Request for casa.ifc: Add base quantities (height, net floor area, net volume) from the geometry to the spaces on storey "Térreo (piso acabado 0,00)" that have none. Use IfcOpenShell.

First a look at what the model holds.

```python
import ifcopenshell
import ifcopenshell.util.element
import ifcopenshell.util.unit

model = ifcopenshell.open("casa.ifc")
print(model.schema)
for unit_type in ("LENGTHUNIT", "AREAUNIT", "VOLUMEUNIT"):
    print(unit_type, ifcopenshell.util.unit.calculate_unit_scale(model, unit_type))
storey = next(s for s in model.by_type("IfcBuildingStorey") if s.Name == "Térreo (piso acabado 0,00)")
spaces = [e for e in ifcopenshell.util.element.get_decomposition(storey) if e.is_a("IfcSpace")]
for e in sorted(spaces, key=lambda e: e.id()):
    print(e.id(), e.is_a(), e.Name, list(ifcopenshell.util.element.get_psets(e, qtos_only=True)), sep=" | ")
```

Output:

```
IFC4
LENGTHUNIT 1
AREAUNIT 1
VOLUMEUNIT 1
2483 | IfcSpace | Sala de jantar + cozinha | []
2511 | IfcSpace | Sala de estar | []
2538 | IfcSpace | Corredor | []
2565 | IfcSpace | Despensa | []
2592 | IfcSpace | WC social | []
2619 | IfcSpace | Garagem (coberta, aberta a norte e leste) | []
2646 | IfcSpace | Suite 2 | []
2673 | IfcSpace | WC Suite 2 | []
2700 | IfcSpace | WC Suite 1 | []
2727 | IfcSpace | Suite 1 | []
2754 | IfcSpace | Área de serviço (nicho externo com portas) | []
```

```python
import ifcopenshell
import ifcopenshell.api.pset
import ifcopenshell.geom
import ifcopenshell.util.element
import ifcopenshell.util.shape
import ifcopenshell.util.unit

model = ifcopenshell.open("casa.ifc")
unit_scale = ifcopenshell.util.unit.calculate_unit_scale(model)
area_scale = ifcopenshell.util.unit.calculate_unit_scale(model, "AREAUNIT")
volume_scale = ifcopenshell.util.unit.calculate_unit_scale(model, "VOLUMEUNIT")
settings = ifcopenshell.geom.settings()

storey = next(s for s in model.by_type("IfcBuildingStorey") if s.Name == "Térreo (piso acabado 0,00)")
spaces = [e for e in ifcopenshell.util.element.get_decomposition(storey) if e.is_a("IfcSpace")]

for e in sorted(spaces, key=lambda e: e.id()):
    if ifcopenshell.util.element.get_psets(e, qtos_only=True, should_inherit=False):
        continue
    # Geometry comes back in metres, in the element's own axes.
    shape = ifcopenshell.geom.create_shape(settings, e)
    values = {
        "Height": ifcopenshell.util.shape.get_z(shape.geometry) / unit_scale,
        "NetFloorArea": ifcopenshell.util.shape.get_footprint_area(shape.geometry) / area_scale,
        "NetVolume": ifcopenshell.util.shape.get_volume(shape.geometry) / volume_scale,
    }
    qto = ifcopenshell.api.pset.add_qto(model, product=e, name="Qto_SpaceBaseQuantities")
    ifcopenshell.api.pset.edit_qto(model, qto=qto, properties=values)
    print(e.id(), {k: round(v, 3) for k, v in values.items()})

model.write("casa_v2.ifc")
```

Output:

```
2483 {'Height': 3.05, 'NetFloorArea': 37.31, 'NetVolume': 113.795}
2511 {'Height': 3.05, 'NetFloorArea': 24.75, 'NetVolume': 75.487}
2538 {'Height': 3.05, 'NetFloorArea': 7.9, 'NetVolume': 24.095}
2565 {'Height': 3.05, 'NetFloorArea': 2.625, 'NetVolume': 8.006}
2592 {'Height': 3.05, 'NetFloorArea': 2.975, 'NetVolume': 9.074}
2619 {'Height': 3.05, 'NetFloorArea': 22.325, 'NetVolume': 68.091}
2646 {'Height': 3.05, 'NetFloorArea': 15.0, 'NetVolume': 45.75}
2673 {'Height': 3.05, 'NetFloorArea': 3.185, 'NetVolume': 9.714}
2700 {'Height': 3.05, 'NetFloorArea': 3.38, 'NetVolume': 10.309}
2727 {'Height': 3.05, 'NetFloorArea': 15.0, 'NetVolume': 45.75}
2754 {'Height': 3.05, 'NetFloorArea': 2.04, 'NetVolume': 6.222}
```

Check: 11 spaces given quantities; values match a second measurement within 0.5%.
